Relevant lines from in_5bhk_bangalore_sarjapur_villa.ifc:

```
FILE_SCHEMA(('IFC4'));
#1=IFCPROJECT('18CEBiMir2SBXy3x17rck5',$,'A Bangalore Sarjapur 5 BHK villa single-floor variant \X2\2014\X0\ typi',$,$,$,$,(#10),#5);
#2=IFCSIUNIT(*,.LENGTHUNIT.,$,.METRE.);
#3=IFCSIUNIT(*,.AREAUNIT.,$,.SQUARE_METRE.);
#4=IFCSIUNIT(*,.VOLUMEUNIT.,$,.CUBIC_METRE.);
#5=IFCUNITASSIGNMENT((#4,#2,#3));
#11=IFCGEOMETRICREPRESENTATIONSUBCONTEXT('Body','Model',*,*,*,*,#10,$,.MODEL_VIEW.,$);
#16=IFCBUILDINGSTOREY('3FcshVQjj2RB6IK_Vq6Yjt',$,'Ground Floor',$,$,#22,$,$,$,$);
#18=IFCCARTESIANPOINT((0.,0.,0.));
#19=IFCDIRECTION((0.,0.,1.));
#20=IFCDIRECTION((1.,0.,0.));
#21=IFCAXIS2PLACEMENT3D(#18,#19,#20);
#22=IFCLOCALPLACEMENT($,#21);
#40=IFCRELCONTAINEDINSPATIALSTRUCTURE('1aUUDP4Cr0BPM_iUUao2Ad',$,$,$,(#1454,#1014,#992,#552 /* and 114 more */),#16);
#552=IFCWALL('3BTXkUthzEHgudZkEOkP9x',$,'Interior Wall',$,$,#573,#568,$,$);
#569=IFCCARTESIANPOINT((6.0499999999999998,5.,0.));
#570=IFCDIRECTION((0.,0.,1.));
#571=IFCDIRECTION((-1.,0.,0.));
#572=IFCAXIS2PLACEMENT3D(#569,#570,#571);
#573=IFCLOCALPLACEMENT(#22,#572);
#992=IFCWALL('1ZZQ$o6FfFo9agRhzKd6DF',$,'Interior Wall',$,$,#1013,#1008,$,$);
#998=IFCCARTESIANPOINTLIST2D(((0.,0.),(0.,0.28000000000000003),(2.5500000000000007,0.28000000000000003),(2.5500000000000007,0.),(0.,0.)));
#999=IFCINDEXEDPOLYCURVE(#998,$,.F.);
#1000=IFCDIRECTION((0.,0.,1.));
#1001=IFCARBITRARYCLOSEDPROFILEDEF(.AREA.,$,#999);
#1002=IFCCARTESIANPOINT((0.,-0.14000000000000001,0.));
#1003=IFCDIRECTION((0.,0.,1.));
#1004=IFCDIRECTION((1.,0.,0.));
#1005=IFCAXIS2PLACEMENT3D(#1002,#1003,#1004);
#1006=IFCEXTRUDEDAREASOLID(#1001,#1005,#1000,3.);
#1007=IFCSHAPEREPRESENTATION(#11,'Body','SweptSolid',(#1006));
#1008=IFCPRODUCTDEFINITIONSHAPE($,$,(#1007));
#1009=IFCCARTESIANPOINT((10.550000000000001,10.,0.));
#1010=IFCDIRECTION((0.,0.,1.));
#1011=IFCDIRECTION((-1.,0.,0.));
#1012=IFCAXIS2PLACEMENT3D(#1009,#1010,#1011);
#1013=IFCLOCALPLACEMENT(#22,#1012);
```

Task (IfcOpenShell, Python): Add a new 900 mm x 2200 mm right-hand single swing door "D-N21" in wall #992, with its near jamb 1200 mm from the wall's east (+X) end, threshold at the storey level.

```python
import numpy as np
import ifcopenshell
import ifcopenshell.api.feature
import ifcopenshell.api.geometry
import ifcopenshell.api.root
import ifcopenshell.api.spatial
import ifcopenshell.geom
import ifcopenshell.util.element
import ifcopenshell.util.placement
import ifcopenshell.util.representation
import ifcopenshell.util.shape
import ifcopenshell.util.unit

model = ifcopenshell.open("in_5bhk_bangalore_sarjapur_villa.ifc")
unit_scale = ifcopenshell.util.unit.calculate_unit_scale(model)
settings = ifcopenshell.geom.settings()


def volume(element):
    """Net volume in cubic metres, openings subtracted."""
    shape = ifcopenshell.geom.create_shape(settings, element)
    return ifcopenshell.util.shape.get_volume(shape.geometry)


wall = model.by_id(992)
storey = ifcopenshell.util.element.get_container(wall, ifc_class="IfcBuildingStorey")
context = ifcopenshell.util.representation.get_context(model, "Model", "Body", "MODEL_VIEW")
before = volume(wall)

width, height, from_end, sill = 0.9, 2.2, 1.2, 0.0  # metres

# The wall runs along its own X axis, and the end named is its -X end.
wall_shape = ifcopenshell.geom.create_shape(settings, wall)
x, y, z = ifcopenshell.util.shape.get_vertices(wall_shape.geometry).T
start = x.min() + from_end
face, thickness = float(y.min()), float(y.max() - y.min())
wall_matrix = ifcopenshell.util.placement.get_local_placement(wall.ObjectPlacement)
level = ifcopenshell.util.placement.get_local_placement(storey.ObjectPlacement)[2, 3]


def in_wall(x, y):
    """Placement at x, y metres in the wall's axes, at sill height."""
    matrix = wall_matrix.copy()
    matrix[:, 3] = wall_matrix @ np.array([x / unit_scale, y / unit_scale, 0.0, 1.0])
    matrix[2, 3] = level + sill / unit_scale
    return matrix


# Opening: a box that overshoots both wall faces by 50 mm.
opening = ifcopenshell.api.root.create_entity(model, ifc_class="IfcOpeningElement", predefined_type="OPENING")
box = ifcopenshell.api.geometry.add_wall_representation(
    model, context=context, length=width, height=height, thickness=thickness + 0.1
)
ifcopenshell.api.geometry.assign_representation(model, product=opening, representation=box)
ifcopenshell.api.geometry.edit_object_placement(model, product=opening, matrix=in_wall(start, face - 0.05), is_si=False)
ifcopenshell.api.feature.add_feature(model, feature=opening, element=wall)

door = ifcopenshell.api.root.create_entity(model, ifc_class="IfcDoor", name="D-N21", predefined_type="DOOR")
door.OverallWidth, door.OverallHeight = width / unit_scale, height / unit_scale
door.OperationType = "SINGLE_SWING_RIGHT"
body = ifcopenshell.api.geometry.add_door_representation(
    model,
    context=context,
    overall_width=door.OverallWidth,
    overall_height=door.OverallHeight,
    operation_type="SINGLE_SWING_RIGHT",
    lining_properties={"LiningDepth": thickness / unit_scale, "ThresholdDepth": thickness / unit_scale},
)
ifcopenshell.api.geometry.assign_representation(model, product=door, representation=body)
ifcopenshell.api.spatial.assign_container(model, products=[door], relating_structure=storey)
ifcopenshell.api.feature.add_filling(model, opening=opening, element=door)

# The lining spans the wall, so the door starts at the wall face.
ifcopenshell.api.geometry.edit_object_placement(model, product=door, matrix=in_wall(start, face), is_si=False)

after = volume(wall)

print(f"wall volume {before:.3f} -> {after:.3f} m3")

model.write("in_5bhk_bangalore_sarjapur_villa_v2.ifc")
```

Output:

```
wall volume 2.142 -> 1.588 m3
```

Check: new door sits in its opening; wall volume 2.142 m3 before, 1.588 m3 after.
